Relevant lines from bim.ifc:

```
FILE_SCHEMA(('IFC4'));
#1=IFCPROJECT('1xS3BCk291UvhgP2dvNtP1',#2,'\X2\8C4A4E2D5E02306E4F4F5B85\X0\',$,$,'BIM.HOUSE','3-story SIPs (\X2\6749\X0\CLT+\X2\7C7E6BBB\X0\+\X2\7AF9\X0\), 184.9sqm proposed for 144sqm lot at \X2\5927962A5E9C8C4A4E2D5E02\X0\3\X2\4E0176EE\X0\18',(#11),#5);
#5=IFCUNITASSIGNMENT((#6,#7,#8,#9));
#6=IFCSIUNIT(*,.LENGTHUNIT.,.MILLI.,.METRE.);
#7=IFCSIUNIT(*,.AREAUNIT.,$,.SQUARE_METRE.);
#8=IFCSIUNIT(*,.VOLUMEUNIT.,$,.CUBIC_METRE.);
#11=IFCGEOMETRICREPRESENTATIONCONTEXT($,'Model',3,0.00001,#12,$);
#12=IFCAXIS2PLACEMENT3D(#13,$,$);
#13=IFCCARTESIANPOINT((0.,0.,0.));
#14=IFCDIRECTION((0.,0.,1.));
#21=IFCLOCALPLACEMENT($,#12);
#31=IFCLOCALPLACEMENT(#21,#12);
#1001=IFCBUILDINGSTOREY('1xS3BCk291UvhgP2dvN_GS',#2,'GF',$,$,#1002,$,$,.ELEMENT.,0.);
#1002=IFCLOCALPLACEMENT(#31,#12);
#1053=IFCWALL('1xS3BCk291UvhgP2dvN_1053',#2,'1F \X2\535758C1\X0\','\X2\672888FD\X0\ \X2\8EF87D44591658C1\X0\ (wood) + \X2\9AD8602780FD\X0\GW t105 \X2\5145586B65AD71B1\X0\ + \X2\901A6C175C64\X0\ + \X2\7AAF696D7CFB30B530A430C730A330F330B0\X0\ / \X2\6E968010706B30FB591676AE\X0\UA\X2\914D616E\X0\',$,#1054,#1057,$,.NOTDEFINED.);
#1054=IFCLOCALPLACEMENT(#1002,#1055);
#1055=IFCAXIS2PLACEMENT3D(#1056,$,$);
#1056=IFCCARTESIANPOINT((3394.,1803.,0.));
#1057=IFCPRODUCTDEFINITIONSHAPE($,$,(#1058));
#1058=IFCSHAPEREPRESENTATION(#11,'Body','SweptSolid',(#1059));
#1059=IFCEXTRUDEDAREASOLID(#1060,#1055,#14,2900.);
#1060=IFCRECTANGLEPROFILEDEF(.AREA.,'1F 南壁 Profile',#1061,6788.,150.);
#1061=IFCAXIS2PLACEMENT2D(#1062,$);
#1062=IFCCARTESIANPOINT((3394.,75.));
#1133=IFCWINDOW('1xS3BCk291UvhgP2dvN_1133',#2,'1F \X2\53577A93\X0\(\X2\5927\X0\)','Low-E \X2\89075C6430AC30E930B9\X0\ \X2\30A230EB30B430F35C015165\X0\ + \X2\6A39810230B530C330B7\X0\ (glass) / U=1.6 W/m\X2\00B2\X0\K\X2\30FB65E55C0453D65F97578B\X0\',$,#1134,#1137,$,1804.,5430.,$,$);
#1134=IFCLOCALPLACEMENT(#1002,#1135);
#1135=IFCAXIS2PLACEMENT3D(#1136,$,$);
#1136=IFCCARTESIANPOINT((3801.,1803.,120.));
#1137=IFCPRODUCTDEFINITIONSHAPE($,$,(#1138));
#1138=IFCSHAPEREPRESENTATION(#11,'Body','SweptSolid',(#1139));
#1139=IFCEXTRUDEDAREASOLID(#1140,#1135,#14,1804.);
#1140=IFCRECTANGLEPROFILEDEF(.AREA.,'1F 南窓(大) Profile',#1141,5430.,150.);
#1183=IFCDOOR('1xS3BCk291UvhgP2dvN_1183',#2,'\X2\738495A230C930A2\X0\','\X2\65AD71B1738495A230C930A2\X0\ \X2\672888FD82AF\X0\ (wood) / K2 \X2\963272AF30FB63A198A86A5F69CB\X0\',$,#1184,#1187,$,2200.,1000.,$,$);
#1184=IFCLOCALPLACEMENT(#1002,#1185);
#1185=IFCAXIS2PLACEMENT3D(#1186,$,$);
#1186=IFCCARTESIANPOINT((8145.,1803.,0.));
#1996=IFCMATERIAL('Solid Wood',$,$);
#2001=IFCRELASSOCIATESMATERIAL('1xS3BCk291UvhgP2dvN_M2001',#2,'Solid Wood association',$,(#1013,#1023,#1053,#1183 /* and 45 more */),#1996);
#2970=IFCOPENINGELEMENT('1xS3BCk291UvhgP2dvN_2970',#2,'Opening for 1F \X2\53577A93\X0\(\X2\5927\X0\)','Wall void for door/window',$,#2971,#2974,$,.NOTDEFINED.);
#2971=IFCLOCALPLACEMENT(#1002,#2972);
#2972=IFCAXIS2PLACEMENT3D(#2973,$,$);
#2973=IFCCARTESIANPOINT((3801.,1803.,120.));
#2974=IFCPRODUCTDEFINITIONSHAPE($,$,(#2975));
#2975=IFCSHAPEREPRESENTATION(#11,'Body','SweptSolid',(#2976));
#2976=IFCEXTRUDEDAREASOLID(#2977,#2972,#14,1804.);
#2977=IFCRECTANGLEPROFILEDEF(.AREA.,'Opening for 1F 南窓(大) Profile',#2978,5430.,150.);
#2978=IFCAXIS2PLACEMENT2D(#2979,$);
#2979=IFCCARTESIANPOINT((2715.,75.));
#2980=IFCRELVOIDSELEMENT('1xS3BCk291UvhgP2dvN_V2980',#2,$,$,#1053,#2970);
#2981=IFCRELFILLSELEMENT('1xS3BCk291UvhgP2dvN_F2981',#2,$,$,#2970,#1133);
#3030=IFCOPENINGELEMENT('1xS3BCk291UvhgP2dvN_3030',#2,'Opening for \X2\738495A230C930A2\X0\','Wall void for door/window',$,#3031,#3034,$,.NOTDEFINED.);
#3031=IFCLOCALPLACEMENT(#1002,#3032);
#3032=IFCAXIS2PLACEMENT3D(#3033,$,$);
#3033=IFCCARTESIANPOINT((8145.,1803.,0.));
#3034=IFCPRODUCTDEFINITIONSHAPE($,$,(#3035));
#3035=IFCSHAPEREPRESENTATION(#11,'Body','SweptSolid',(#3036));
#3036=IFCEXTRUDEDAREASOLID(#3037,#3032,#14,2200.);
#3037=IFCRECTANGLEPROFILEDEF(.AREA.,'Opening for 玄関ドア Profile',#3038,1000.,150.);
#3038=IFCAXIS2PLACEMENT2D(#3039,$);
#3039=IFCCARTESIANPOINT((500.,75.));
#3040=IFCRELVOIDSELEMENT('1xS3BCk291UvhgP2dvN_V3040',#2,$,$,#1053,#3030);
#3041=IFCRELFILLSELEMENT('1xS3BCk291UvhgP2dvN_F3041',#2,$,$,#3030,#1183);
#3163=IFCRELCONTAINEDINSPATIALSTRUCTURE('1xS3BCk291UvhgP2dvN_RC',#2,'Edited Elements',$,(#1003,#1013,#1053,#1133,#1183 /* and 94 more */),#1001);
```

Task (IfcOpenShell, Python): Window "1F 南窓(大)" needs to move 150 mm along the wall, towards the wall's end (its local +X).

```python
import ifcopenshell
import ifcopenshell.api.geometry
import ifcopenshell.util.placement
import ifcopenshell.util.unit

model = ifcopenshell.open("bim.ifc")
unit_scale = ifcopenshell.util.unit.calculate_unit_scale(model)

window = model.by_id(1133)
opening = window.FillsVoids[0].RelatingOpeningElement
wall = opening.VoidsElements[0].RelatingBuildingElement

wall_matrix = ifcopenshell.util.placement.get_local_placement(wall.ObjectPlacement)
shift = wall_matrix[:3, 0] * 0.15 / unit_scale
before = ifcopenshell.util.placement.get_local_placement(window.ObjectPlacement)[:3, 3].copy()

# The window is not placed relative to its opening, so move both.
for product in (opening, window):
    matrix = ifcopenshell.util.placement.get_local_placement(product.ObjectPlacement)
    matrix[:3, 3] += shift
    ifcopenshell.api.geometry.edit_object_placement(model, product=product, matrix=matrix, is_si=False)

after = ifcopenshell.util.placement.get_local_placement(window.ObjectPlacement)[:3, 3]
print("window moved by", (after - before).round(3) + 0.0)

model.write("bim_edited.ifc")
```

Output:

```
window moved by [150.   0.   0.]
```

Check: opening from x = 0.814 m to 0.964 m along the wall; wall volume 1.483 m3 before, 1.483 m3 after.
